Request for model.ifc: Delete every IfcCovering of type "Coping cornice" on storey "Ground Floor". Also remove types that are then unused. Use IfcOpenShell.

First a look at what the model holds.

```python
import ifcopenshell
import ifcopenshell.util.element

model = ifcopenshell.open("model.ifc")
print(model.schema)
storey = next(s for s in model.by_type("IfcBuildingStorey") if s.Name == "Ground Floor")
coverings = [e for e in ifcopenshell.util.element.get_decomposition(storey) if e.is_a("IfcCovering")]
seen = {}
for e in coverings:
    element_type = ifcopenshell.util.element.get_type(e)
    name = element_type.Name if element_type not in (None, e) else None
    seen[name] = seen.get(name, 0) + 1
for name, count in sorted(seen.items(), key=str):
    print(count, "x", name)
```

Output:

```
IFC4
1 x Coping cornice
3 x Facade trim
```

```python
import ifcopenshell
import ifcopenshell.api.root
import ifcopenshell.util.element

model = ifcopenshell.open("model.ifc")

storey = next(s for s in model.by_type("IfcBuildingStorey") if s.Name == "Ground Floor")
coverings = [e for e in ifcopenshell.util.element.get_decomposition(storey) if e.is_a("IfcCovering")]
targets = [e for e in coverings if (t := ifcopenshell.util.element.get_type(e)) not in (None, e) and t.Name == "Coping cornice"]
types = {ifcopenshell.util.element.get_type(e) for e in targets} - {None, *targets}

for e in targets:
    ifcopenshell.api.root.remove_product(model, product=e)
print(len(targets), "removed")

unused = [t for t in types if not ifcopenshell.util.element.get_types(t)]
for t in unused:
    ifcopenshell.api.root.remove_product(model, product=t)
print(len(unused), "unused types removed")

model.write("model_rev.ifc")
```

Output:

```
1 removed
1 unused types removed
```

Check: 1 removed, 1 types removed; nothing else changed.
